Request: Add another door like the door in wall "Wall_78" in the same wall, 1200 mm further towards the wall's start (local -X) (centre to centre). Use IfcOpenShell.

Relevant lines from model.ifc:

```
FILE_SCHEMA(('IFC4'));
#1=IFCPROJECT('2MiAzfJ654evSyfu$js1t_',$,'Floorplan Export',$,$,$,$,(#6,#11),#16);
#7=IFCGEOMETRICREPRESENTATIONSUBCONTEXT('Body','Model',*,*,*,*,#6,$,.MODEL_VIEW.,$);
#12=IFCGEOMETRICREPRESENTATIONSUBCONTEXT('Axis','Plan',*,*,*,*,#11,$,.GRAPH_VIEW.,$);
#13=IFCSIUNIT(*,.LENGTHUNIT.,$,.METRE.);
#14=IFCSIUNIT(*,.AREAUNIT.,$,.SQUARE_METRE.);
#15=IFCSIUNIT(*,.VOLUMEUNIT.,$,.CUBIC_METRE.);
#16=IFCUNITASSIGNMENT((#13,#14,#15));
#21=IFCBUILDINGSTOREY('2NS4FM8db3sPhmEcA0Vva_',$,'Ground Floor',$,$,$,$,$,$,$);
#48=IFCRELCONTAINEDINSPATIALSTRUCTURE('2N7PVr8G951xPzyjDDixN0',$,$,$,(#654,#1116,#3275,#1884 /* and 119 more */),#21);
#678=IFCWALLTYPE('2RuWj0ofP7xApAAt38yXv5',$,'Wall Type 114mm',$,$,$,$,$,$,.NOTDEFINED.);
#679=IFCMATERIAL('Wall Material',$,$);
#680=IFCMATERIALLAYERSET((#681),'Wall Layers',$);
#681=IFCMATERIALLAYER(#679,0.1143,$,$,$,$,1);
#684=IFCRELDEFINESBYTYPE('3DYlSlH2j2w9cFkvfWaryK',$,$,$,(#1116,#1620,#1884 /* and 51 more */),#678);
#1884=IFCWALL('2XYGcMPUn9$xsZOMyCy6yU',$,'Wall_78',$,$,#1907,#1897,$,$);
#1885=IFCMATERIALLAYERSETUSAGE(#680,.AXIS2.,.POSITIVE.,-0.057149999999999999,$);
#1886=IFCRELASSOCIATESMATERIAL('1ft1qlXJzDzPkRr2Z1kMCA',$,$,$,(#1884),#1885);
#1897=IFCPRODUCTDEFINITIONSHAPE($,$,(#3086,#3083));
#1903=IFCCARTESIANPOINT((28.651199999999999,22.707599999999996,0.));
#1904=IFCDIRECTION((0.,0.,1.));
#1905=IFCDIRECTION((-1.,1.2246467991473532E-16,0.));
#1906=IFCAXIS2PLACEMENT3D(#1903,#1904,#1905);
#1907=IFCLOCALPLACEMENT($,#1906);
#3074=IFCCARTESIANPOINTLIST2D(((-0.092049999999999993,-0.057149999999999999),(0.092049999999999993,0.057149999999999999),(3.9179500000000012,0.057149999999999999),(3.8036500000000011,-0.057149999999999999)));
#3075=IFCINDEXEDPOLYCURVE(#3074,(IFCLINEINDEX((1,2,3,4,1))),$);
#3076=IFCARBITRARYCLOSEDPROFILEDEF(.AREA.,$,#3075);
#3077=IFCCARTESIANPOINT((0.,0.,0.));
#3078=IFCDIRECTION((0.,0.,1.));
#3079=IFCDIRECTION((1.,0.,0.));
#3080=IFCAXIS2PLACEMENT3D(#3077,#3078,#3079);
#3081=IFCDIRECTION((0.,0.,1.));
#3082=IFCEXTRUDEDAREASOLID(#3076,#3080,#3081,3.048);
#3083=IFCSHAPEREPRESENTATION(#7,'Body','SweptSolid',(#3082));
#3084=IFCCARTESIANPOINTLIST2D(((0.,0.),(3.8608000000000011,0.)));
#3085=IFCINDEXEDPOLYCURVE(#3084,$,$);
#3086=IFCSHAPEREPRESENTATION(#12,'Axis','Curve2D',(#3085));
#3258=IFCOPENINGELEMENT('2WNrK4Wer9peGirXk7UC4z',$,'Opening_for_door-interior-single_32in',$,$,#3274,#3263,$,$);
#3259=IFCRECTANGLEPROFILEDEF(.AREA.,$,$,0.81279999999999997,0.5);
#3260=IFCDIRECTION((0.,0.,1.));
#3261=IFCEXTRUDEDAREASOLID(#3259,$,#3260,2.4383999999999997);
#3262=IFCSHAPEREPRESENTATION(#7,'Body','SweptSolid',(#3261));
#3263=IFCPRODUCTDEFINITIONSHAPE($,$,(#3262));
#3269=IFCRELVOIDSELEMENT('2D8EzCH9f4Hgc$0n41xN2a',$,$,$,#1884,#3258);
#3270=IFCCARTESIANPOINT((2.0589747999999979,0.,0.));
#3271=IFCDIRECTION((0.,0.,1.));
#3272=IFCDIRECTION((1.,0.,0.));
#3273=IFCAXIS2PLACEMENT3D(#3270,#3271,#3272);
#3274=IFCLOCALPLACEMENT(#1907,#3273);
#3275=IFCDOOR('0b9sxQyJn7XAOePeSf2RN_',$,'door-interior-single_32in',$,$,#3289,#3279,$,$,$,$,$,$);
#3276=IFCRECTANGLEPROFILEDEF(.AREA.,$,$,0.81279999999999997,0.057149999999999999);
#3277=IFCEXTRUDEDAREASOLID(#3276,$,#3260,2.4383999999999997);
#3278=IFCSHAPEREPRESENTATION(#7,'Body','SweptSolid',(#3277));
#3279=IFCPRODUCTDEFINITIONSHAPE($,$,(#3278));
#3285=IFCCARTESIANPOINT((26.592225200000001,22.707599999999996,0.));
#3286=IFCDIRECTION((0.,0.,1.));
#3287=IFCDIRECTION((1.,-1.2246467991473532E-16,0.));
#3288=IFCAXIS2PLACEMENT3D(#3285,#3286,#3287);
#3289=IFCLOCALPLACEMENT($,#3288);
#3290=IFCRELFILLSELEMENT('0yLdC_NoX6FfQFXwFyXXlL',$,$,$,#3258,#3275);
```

```python
import ifcopenshell
import ifcopenshell.api.feature
import ifcopenshell.api.geometry
import ifcopenshell.api.root
import ifcopenshell.geom
import ifcopenshell.util.element
import ifcopenshell.util.placement
import ifcopenshell.util.shape
import ifcopenshell.util.unit

model = ifcopenshell.open("model.ifc")
unit_scale = ifcopenshell.util.unit.calculate_unit_scale(model)
settings = ifcopenshell.geom.settings()


def volume(element):
    """Net volume in cubic metres, openings subtracted."""
    shape = ifcopenshell.geom.create_shape(settings, element)
    return ifcopenshell.util.shape.get_volume(shape.geometry)


door = model.by_guid("0b9sxQyJn7XAOePeSf2RN_")
opening = door.FillsVoids[0].RelatingOpeningElement
wall = opening.VoidsElements[0].RelatingBuildingElement
before = volume(wall)
shift = ifcopenshell.util.placement.get_local_placement(wall.ObjectPlacement)[:3, 0] * -1.2 / unit_scale

# copy_class copies the void relationship, type, container and properties, but no geometry.
new_opening = ifcopenshell.api.root.copy_class(model, product=opening)
new_opening.Representation = ifcopenshell.util.element.copy_deep(
    model, opening.Representation, exclude=["IfcGeometricRepresentationContext", "IfcRepresentationMap"]
)
new_door = ifcopenshell.api.root.copy_class(model, product=door)
new_door.Representation = ifcopenshell.util.element.copy_deep(
    model, door.Representation, exclude=["IfcGeometricRepresentationContext", "IfcRepresentationMap"]
)
ifcopenshell.api.feature.add_filling(model, opening=new_opening, element=new_door)

for old, new in ((opening, new_opening), (door, new_door)):
    matrix = ifcopenshell.util.placement.get_local_placement(old.ObjectPlacement)
    matrix[:3, 3] += shift
    ifcopenshell.api.geometry.edit_object_placement(model, product=new, matrix=matrix, is_si=False)

after = volume(wall)

print(f"wall volume {before:.3f} -> {after:.3f} m3")

model.write("model_rev.ifc")
```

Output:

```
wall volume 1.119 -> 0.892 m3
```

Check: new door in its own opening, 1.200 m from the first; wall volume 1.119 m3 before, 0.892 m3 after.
